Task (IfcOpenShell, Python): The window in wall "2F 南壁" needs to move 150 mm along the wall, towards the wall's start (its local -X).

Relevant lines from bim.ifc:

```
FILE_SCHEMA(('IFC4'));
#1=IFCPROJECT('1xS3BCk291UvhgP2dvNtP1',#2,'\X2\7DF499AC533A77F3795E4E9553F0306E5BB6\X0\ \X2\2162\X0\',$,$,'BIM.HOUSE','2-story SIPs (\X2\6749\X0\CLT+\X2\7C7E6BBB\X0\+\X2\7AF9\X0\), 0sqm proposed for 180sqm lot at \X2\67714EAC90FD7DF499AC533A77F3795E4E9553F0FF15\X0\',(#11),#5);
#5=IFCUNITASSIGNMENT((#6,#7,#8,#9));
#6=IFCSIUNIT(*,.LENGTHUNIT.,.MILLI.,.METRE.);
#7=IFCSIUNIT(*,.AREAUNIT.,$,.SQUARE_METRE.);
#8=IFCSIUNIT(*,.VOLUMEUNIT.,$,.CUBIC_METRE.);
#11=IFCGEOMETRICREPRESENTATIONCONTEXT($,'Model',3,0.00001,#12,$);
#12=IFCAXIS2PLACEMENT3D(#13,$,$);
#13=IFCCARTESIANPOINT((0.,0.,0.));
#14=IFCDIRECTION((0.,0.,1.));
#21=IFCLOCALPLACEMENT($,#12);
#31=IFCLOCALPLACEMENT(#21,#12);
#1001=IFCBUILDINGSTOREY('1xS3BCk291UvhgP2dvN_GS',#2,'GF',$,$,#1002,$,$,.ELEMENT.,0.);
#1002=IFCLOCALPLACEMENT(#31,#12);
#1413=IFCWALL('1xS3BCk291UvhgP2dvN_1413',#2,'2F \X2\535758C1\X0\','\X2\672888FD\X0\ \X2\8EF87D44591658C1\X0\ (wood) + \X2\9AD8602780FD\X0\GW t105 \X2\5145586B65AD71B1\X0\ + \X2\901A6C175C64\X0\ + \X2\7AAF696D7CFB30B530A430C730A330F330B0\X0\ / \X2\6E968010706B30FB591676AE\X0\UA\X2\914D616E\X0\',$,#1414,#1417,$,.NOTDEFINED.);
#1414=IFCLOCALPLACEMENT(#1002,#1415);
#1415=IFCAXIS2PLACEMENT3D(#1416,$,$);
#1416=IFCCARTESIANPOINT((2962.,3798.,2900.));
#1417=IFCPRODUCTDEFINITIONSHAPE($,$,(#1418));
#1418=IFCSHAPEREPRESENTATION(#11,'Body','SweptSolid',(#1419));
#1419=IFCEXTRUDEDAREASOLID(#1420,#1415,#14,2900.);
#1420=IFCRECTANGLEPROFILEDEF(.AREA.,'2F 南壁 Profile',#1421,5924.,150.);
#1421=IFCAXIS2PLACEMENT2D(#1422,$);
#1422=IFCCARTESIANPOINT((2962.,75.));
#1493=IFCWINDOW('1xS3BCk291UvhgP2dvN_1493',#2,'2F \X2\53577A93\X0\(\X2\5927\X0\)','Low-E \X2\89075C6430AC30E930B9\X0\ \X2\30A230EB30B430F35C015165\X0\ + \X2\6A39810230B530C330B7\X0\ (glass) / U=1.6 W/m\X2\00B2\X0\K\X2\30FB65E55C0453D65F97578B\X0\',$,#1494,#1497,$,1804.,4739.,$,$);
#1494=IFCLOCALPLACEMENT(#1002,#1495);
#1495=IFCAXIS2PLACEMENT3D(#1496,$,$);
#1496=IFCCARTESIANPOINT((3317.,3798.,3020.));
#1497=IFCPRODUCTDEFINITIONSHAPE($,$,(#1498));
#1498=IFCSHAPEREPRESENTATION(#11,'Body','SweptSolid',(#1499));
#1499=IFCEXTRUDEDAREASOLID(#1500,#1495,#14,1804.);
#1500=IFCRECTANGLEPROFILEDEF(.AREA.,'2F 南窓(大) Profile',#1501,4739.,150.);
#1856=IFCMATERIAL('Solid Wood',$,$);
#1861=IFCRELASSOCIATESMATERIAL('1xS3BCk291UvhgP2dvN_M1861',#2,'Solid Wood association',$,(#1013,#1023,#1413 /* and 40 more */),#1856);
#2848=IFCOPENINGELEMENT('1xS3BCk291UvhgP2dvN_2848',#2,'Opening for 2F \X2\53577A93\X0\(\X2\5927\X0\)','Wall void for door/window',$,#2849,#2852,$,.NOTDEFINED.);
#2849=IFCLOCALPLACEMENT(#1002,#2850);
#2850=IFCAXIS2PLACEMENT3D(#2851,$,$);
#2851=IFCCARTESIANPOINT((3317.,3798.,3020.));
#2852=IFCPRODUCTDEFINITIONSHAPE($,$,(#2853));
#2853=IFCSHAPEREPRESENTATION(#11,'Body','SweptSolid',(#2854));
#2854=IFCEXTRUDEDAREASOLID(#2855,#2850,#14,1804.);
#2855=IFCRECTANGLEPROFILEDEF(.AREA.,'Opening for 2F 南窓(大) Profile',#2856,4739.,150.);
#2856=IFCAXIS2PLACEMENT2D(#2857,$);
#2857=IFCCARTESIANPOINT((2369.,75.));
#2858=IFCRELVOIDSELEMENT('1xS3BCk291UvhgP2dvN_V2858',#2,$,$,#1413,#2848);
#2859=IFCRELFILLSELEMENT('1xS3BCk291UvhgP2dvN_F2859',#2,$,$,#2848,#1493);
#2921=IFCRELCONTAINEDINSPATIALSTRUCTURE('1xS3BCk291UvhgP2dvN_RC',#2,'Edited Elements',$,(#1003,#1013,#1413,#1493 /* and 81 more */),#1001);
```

```python
import ifcopenshell
import ifcopenshell.api.geometry
import ifcopenshell.util.placement

model = ifcopenshell.open("bim.ifc")

window = model.by_guid("1xS3BCk291UvhgP2dvN_1493")
opening = window.FillsVoids[0].RelatingOpeningElement
wall = opening.VoidsElements[0].RelatingBuildingElement

wall_matrix = ifcopenshell.util.placement.get_local_placement(wall.ObjectPlacement)
shift = wall_matrix[:3, 0] * -150.0
before = ifcopenshell.util.placement.get_local_placement(window.ObjectPlacement)[:3, 3].copy()

# The window is not placed relative to its opening, so move both.
for product in (opening, window):
    matrix = ifcopenshell.util.placement.get_local_placement(product.ObjectPlacement)
    matrix[:3, 3] += shift
    ifcopenshell.api.geometry.edit_object_placement(model, product=product, matrix=matrix, is_si=False)

after = ifcopenshell.util.placement.get_local_placement(window.ObjectPlacement)[:3, 3]
print("window moved by", (after - before).round(3) + 0.0)

model.write("bim_updated.ifc")
```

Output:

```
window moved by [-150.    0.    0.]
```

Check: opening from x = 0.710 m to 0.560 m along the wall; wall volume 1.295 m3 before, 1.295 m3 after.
